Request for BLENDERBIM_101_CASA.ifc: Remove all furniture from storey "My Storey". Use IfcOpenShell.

First a look at what the model holds.

```python
import ifcopenshell
import ifcopenshell.util.element

model = ifcopenshell.open("BLENDERBIM_101_CASA.ifc")
print(model.schema)
storey = next(s for s in model.by_type("IfcBuildingStorey") if s.Name == "My Storey")
furniture = [e for e in ifcopenshell.util.element.get_decomposition(storey) if e.is_a("IfcFurnishingElement")]
seen = {}
for e in furniture:
    element_type = ifcopenshell.util.element.get_type(e)
    name = element_type.Name if element_type not in (None, e) else None
    seen[name] = seen.get(name, 0) + 1
for name, count in sorted(seen.items(), key=str):
    print(count, "x", name)
```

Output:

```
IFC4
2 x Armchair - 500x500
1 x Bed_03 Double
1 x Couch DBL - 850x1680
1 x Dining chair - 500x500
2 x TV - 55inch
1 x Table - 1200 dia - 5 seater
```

```python
import ifcopenshell
import ifcopenshell.api.root
import ifcopenshell.util.element

model = ifcopenshell.open("BLENDERBIM_101_CASA.ifc")

storey = next(s for s in model.by_type("IfcBuildingStorey") if s.Name == "My Storey")
furniture = [e for e in ifcopenshell.util.element.get_decomposition(storey) if e.is_a("IfcFurnishingElement")]

for e in furniture:
    ifcopenshell.api.root.remove_product(model, product=e)
print(len(furniture), "removed")

model.write("BLENDERBIM_101_CASA_rev.ifc")
```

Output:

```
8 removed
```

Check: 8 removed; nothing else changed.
